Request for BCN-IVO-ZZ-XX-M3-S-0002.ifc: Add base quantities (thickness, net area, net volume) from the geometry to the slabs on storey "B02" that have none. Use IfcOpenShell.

First a look at what the model holds.

```python
import ifcopenshell
import ifcopenshell.util.element
import ifcopenshell.util.unit

model = ifcopenshell.open("BCN-IVO-ZZ-XX-M3-S-0002.ifc")
print(model.schema)
for unit_type in ("LENGTHUNIT", "AREAUNIT", "VOLUMEUNIT"):
    print(unit_type, ifcopenshell.util.unit.calculate_unit_scale(model, unit_type))
storey = next(s for s in model.by_type("IfcBuildingStorey") if s.Name == "B02")
slabs = [e for e in ifcopenshell.util.element.get_decomposition(storey) if e.is_a("IfcSlab")]
for e in sorted(slabs, key=lambda e: e.id()):
    print(e.id(), e.is_a(), e.Name, list(ifcopenshell.util.element.get_psets(e, qtos_only=True)), sep=" | ")
```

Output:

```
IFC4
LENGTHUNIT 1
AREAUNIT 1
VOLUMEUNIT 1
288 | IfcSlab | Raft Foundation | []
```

```python
import ifcopenshell
import ifcopenshell.api.pset
import ifcopenshell.geom
import ifcopenshell.util.element
import ifcopenshell.util.shape
import ifcopenshell.util.unit

model = ifcopenshell.open("BCN-IVO-ZZ-XX-M3-S-0002.ifc")
unit_scale = ifcopenshell.util.unit.calculate_unit_scale(model)
area_scale = ifcopenshell.util.unit.calculate_unit_scale(model, "AREAUNIT")
volume_scale = ifcopenshell.util.unit.calculate_unit_scale(model, "VOLUMEUNIT")
settings = ifcopenshell.geom.settings()

storey = next(s for s in model.by_type("IfcBuildingStorey") if s.Name == "B02")
slabs = [e for e in ifcopenshell.util.element.get_decomposition(storey) if e.is_a("IfcSlab")]

for e in sorted(slabs, key=lambda e: e.id()):
    if ifcopenshell.util.element.get_psets(e, qtos_only=True, should_inherit=False):
        continue
    # Geometry comes back in metres, in the element's own axes.
    shape = ifcopenshell.geom.create_shape(settings, e)
    values = {
        "Width": ifcopenshell.util.shape.get_z(shape.geometry) / unit_scale,
        "NetArea": ifcopenshell.util.shape.get_footprint_area(shape.geometry) / area_scale,
        "NetVolume": ifcopenshell.util.shape.get_volume(shape.geometry) / volume_scale,
    }
    qto = ifcopenshell.api.pset.add_qto(model, product=e, name="Qto_SlabBaseQuantities")
    ifcopenshell.api.pset.edit_qto(model, qto=qto, properties=values)
    print(e.id(), {k: round(v, 3) for k, v in values.items()})

model.write("BCN-IVO-ZZ-XX-M3-S-0002_updated.ifc")
```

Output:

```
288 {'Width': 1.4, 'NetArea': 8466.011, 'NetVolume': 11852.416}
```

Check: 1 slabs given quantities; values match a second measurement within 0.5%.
